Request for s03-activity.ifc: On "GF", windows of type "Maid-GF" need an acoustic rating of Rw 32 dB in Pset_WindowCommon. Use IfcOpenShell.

First a look at what the model holds.

```python
import ifcopenshell
import ifcopenshell.util.element

model = ifcopenshell.open("s03-activity.ifc")
print(model.schema)
storey = next(s for s in model.by_type("IfcBuildingStorey") if s.Name == "GF")
windows = [e for e in ifcopenshell.util.element.get_decomposition(storey) if e.is_a("IfcWindow")]
seen = {}
for e in windows:
    element_type = ifcopenshell.util.element.get_type(e)
    key = (element_type.Name if element_type != e and element_type else None, ifcopenshell.util.element.get_pset(e, "Pset_WindowCommon", "AcousticRating"))
    seen[key] = seen.get(key, 0) + 1
for (name, value), count in sorted(seen.items(), key=str):
    print(count, "x", name, "|", value)
```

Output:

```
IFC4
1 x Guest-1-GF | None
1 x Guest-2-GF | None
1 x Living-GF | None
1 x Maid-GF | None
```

```python
import ifcopenshell
import ifcopenshell.api.pset
import ifcopenshell.util.element

model = ifcopenshell.open("s03-activity.ifc")

storey = next(s for s in model.by_type("IfcBuildingStorey") if s.Name == "GF")
windows = [e for e in ifcopenshell.util.element.get_decomposition(storey) if e.is_a("IfcWindow")]

count = 0
for e in windows:
    element_type = ifcopenshell.util.element.get_type(e)
    if element_type in (None, e) or element_type.Name != "Maid-GF":
        continue
    # add_pset returns the element's existing set when there is one.
    pset = ifcopenshell.api.pset.add_pset(model, product=e, name="Pset_WindowCommon")
    ifcopenshell.api.pset.edit_pset(model, pset=pset, properties={"AcousticRating": "Rw 32 dB"})
    count += 1

print(count, "windows updated")

model.write("s03-activity_v2.ifc")
```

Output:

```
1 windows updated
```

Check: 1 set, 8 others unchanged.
